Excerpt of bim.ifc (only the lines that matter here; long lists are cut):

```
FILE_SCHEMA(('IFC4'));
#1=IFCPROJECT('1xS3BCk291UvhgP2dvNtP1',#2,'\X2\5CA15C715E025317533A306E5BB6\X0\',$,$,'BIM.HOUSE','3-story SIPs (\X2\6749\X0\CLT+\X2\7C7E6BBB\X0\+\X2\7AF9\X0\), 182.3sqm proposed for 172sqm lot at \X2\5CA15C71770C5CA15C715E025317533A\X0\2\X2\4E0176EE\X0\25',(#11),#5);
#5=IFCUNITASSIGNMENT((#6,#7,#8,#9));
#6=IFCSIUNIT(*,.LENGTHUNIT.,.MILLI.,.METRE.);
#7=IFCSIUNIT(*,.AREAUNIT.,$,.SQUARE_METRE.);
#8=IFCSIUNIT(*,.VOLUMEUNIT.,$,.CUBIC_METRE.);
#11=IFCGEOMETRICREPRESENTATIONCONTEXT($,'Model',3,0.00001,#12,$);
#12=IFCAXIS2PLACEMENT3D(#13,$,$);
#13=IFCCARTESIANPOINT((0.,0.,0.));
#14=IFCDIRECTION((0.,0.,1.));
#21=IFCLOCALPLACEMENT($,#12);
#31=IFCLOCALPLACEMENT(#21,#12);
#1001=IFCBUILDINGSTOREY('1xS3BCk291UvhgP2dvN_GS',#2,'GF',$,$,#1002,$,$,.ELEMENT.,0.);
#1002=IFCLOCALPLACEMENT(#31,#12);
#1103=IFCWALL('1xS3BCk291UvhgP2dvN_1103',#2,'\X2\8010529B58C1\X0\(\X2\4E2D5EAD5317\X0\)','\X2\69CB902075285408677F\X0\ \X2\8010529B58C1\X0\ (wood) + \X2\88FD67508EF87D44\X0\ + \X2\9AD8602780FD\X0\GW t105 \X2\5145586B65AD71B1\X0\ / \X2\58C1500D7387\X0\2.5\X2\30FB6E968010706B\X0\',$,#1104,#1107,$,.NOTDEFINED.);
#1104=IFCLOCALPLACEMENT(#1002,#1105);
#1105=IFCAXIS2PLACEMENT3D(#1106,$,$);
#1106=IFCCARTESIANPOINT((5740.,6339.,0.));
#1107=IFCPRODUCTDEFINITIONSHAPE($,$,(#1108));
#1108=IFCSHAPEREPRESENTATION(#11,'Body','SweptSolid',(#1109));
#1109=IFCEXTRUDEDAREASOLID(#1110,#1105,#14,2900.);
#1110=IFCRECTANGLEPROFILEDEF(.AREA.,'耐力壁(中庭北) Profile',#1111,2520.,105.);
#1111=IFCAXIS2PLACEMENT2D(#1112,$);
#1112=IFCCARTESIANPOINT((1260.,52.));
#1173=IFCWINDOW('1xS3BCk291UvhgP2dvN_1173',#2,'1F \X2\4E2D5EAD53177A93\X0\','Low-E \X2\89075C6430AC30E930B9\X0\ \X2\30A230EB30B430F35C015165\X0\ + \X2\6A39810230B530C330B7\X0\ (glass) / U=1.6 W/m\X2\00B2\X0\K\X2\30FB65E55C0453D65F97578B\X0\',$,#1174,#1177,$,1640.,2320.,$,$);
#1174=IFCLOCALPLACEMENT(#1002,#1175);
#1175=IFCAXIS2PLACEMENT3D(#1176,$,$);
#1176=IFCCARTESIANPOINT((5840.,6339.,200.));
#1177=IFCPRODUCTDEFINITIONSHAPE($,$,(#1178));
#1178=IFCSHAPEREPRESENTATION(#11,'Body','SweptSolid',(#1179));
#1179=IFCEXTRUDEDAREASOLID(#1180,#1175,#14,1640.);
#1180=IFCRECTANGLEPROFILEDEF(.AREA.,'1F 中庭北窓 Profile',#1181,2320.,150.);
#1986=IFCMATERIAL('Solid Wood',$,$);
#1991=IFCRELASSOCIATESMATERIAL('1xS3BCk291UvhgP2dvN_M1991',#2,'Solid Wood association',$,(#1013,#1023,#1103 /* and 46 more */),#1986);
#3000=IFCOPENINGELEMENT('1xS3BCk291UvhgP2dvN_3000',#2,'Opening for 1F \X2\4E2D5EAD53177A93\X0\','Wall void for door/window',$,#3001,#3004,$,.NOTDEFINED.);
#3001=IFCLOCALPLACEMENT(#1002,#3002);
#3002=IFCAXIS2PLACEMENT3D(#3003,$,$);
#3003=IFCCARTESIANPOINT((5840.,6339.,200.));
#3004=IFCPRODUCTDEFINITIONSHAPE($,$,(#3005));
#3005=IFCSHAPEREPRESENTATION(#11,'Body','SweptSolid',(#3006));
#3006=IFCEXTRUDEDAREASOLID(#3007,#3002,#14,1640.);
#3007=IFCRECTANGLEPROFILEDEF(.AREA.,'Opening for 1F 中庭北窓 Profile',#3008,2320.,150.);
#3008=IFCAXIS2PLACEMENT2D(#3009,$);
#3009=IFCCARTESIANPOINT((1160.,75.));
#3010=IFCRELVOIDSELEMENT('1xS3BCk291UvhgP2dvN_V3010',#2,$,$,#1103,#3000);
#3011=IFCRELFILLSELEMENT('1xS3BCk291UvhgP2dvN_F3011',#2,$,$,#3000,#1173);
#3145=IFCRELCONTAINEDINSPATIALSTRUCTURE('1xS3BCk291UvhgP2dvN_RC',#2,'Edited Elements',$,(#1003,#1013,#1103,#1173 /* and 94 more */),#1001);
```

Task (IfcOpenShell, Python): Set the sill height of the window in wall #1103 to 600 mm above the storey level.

```python
import numpy as np
import ifcopenshell
import ifcopenshell.api.geometry
import ifcopenshell.geom
import ifcopenshell.util.element
import ifcopenshell.util.placement
import ifcopenshell.util.shape
import ifcopenshell.util.unit

model = ifcopenshell.open("bim.ifc")
unit_scale = ifcopenshell.util.unit.calculate_unit_scale(model)

window = model.by_guid("1xS3BCk291UvhgP2dvN_1173")
opening = window.FillsVoids[0].RelatingOpeningElement
storey = ifcopenshell.util.element.get_container(window, ifc_class="IfcBuildingStorey")
level = ifcopenshell.util.placement.get_local_placement(storey.ObjectPlacement)[2, 3]

# The opening's origin need not be at the sill, so measure its lowest point.
shape = ifcopenshell.geom.create_shape(ifcopenshell.geom.settings(), opening)
bottom = ifcopenshell.util.shape.get_shape_bottom_elevation(shape, shape.geometry) / unit_scale
dz = level + 0.6 / unit_scale - bottom

shift = np.array([0.0, 0.0, dz])
# The window is not placed relative to its opening, so move both.
for product in (opening, window):
    matrix = ifcopenshell.util.placement.get_local_placement(product.ObjectPlacement)
    matrix[:3, 3] += shift
    ifcopenshell.api.geometry.edit_object_placement(model, product=product, matrix=matrix, is_si=False)

print(f"moved by {dz * unit_scale:+.3f} m")

model.write("bim_edited.ifc")
```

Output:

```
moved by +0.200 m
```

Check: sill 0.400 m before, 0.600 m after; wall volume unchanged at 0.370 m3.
